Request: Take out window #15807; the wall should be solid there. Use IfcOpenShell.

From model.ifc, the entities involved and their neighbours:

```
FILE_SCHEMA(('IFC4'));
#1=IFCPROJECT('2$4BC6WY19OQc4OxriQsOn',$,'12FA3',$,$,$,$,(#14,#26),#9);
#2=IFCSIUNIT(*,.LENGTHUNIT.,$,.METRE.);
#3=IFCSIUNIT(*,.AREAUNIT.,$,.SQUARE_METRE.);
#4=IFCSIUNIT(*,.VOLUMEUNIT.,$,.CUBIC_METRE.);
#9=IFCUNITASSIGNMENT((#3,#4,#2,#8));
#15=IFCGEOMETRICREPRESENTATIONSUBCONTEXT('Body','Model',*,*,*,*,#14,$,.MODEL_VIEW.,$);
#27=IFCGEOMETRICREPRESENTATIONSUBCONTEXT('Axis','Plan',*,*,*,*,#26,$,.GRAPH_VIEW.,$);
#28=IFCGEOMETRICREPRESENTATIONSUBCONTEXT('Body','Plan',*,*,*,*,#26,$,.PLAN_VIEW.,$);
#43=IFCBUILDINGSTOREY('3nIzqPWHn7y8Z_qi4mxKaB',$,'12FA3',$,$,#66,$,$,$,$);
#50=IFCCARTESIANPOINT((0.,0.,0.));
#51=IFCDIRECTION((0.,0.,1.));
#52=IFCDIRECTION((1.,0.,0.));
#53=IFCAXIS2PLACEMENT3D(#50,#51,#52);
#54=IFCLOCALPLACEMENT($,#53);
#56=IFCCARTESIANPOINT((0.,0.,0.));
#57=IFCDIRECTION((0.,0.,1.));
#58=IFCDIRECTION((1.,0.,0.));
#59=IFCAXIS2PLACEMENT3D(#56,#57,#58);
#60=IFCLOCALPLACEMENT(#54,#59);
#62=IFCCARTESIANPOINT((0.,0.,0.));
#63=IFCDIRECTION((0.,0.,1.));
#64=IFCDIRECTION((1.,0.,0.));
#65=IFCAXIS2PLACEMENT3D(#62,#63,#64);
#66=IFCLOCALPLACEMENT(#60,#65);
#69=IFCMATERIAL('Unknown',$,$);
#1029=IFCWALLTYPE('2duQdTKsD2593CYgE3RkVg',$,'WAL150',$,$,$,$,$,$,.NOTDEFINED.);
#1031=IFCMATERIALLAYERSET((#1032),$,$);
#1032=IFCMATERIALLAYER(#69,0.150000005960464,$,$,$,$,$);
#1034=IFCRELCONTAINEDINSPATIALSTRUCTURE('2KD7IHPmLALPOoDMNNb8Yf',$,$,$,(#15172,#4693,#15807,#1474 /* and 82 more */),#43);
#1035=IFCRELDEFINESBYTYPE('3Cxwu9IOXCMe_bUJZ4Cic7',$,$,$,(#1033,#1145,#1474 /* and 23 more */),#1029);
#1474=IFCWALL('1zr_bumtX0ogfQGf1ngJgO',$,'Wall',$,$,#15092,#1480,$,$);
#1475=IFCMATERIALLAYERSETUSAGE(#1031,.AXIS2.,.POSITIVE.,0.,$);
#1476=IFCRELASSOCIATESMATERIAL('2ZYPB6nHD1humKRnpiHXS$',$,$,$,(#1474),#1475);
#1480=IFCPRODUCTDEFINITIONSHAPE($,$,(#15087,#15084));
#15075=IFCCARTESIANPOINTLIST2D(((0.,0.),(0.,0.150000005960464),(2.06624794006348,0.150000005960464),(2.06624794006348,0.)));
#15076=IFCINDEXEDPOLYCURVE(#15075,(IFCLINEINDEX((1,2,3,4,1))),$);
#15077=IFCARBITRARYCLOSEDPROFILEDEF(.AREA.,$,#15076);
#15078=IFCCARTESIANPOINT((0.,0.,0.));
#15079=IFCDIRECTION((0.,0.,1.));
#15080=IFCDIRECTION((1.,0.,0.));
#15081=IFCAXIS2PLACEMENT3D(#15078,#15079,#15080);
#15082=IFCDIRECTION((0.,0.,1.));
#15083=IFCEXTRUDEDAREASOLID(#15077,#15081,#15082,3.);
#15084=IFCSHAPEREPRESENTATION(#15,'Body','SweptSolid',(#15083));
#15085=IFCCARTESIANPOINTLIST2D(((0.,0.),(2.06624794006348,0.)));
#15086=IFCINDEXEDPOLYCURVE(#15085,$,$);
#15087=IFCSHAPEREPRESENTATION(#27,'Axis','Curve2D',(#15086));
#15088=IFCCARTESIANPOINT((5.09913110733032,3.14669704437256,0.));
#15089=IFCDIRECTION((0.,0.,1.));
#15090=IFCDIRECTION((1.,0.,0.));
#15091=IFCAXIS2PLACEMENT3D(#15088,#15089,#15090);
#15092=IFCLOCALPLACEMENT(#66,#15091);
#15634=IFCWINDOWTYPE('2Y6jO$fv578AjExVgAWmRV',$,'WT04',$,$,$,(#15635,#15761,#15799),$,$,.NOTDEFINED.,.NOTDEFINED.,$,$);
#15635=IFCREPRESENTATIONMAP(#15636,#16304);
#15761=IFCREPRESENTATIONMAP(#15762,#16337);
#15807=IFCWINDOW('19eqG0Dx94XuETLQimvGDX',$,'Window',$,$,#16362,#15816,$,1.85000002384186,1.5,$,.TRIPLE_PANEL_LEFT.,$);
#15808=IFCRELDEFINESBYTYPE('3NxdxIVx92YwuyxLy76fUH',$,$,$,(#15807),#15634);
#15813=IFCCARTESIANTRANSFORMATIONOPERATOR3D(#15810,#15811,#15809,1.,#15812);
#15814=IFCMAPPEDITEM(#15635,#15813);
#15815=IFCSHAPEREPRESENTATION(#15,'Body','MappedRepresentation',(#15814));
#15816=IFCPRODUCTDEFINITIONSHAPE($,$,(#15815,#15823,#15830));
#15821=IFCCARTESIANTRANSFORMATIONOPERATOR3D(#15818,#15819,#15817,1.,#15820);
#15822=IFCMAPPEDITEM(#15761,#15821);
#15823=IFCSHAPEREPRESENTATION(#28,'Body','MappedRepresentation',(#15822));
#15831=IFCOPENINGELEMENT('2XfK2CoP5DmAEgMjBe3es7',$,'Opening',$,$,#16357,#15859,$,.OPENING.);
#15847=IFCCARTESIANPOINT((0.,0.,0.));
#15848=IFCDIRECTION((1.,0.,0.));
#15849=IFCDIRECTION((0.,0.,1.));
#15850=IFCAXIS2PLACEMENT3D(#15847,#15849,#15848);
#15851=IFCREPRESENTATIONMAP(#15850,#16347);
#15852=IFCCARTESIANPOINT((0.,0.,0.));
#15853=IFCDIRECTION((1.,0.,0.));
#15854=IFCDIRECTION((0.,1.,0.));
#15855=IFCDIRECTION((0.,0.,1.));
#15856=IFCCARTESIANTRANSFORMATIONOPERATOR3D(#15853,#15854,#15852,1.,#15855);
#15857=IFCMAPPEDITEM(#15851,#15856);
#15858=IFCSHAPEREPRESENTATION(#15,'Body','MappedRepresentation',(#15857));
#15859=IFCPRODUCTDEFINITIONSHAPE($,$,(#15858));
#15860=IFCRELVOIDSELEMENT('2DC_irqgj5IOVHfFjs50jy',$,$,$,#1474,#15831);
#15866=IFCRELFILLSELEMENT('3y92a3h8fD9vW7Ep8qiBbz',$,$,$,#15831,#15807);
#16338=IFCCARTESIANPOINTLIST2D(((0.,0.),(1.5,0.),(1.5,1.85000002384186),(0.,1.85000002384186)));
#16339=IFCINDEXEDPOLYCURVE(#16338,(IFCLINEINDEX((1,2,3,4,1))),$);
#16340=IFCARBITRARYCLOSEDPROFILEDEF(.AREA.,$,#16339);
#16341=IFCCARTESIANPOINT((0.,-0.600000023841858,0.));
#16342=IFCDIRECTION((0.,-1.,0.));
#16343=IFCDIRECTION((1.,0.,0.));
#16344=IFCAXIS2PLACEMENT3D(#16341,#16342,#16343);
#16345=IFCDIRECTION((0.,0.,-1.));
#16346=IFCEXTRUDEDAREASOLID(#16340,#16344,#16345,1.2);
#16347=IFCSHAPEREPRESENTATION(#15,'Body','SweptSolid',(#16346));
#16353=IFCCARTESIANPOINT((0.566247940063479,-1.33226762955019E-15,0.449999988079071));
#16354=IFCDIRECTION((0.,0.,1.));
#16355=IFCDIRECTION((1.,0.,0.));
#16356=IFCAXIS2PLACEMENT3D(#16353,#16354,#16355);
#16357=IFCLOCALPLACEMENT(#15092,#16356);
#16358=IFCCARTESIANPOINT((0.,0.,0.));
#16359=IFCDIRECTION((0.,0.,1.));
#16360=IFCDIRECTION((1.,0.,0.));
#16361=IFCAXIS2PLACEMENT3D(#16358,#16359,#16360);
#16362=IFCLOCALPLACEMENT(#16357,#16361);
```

```python
import ifcopenshell
import ifcopenshell.api.feature
import ifcopenshell.api.root
import ifcopenshell.geom
import ifcopenshell.util.shape

model = ifcopenshell.open("model.ifc")
settings = ifcopenshell.geom.settings()


def volume(element):
    """Net volume in cubic metres, openings subtracted."""
    shape = ifcopenshell.geom.create_shape(settings, element)
    return ifcopenshell.util.shape.get_volume(shape.geometry)


window = model.by_guid("19eqG0Dx94XuETLQimvGDX")
opening = window.FillsVoids[0].RelatingOpeningElement
wall = opening.VoidsElements[0].RelatingBuildingElement
before = volume(wall)

ifcopenshell.api.root.remove_product(model, product=window)
ifcopenshell.api.feature.remove_feature(model, feature=opening)

after = volume(wall)

print(f"wall volume {before:.3f} -> {after:.3f} m3")

model.write("model_edited.ifc")
```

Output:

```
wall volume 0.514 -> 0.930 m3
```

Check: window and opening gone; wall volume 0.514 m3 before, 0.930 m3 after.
